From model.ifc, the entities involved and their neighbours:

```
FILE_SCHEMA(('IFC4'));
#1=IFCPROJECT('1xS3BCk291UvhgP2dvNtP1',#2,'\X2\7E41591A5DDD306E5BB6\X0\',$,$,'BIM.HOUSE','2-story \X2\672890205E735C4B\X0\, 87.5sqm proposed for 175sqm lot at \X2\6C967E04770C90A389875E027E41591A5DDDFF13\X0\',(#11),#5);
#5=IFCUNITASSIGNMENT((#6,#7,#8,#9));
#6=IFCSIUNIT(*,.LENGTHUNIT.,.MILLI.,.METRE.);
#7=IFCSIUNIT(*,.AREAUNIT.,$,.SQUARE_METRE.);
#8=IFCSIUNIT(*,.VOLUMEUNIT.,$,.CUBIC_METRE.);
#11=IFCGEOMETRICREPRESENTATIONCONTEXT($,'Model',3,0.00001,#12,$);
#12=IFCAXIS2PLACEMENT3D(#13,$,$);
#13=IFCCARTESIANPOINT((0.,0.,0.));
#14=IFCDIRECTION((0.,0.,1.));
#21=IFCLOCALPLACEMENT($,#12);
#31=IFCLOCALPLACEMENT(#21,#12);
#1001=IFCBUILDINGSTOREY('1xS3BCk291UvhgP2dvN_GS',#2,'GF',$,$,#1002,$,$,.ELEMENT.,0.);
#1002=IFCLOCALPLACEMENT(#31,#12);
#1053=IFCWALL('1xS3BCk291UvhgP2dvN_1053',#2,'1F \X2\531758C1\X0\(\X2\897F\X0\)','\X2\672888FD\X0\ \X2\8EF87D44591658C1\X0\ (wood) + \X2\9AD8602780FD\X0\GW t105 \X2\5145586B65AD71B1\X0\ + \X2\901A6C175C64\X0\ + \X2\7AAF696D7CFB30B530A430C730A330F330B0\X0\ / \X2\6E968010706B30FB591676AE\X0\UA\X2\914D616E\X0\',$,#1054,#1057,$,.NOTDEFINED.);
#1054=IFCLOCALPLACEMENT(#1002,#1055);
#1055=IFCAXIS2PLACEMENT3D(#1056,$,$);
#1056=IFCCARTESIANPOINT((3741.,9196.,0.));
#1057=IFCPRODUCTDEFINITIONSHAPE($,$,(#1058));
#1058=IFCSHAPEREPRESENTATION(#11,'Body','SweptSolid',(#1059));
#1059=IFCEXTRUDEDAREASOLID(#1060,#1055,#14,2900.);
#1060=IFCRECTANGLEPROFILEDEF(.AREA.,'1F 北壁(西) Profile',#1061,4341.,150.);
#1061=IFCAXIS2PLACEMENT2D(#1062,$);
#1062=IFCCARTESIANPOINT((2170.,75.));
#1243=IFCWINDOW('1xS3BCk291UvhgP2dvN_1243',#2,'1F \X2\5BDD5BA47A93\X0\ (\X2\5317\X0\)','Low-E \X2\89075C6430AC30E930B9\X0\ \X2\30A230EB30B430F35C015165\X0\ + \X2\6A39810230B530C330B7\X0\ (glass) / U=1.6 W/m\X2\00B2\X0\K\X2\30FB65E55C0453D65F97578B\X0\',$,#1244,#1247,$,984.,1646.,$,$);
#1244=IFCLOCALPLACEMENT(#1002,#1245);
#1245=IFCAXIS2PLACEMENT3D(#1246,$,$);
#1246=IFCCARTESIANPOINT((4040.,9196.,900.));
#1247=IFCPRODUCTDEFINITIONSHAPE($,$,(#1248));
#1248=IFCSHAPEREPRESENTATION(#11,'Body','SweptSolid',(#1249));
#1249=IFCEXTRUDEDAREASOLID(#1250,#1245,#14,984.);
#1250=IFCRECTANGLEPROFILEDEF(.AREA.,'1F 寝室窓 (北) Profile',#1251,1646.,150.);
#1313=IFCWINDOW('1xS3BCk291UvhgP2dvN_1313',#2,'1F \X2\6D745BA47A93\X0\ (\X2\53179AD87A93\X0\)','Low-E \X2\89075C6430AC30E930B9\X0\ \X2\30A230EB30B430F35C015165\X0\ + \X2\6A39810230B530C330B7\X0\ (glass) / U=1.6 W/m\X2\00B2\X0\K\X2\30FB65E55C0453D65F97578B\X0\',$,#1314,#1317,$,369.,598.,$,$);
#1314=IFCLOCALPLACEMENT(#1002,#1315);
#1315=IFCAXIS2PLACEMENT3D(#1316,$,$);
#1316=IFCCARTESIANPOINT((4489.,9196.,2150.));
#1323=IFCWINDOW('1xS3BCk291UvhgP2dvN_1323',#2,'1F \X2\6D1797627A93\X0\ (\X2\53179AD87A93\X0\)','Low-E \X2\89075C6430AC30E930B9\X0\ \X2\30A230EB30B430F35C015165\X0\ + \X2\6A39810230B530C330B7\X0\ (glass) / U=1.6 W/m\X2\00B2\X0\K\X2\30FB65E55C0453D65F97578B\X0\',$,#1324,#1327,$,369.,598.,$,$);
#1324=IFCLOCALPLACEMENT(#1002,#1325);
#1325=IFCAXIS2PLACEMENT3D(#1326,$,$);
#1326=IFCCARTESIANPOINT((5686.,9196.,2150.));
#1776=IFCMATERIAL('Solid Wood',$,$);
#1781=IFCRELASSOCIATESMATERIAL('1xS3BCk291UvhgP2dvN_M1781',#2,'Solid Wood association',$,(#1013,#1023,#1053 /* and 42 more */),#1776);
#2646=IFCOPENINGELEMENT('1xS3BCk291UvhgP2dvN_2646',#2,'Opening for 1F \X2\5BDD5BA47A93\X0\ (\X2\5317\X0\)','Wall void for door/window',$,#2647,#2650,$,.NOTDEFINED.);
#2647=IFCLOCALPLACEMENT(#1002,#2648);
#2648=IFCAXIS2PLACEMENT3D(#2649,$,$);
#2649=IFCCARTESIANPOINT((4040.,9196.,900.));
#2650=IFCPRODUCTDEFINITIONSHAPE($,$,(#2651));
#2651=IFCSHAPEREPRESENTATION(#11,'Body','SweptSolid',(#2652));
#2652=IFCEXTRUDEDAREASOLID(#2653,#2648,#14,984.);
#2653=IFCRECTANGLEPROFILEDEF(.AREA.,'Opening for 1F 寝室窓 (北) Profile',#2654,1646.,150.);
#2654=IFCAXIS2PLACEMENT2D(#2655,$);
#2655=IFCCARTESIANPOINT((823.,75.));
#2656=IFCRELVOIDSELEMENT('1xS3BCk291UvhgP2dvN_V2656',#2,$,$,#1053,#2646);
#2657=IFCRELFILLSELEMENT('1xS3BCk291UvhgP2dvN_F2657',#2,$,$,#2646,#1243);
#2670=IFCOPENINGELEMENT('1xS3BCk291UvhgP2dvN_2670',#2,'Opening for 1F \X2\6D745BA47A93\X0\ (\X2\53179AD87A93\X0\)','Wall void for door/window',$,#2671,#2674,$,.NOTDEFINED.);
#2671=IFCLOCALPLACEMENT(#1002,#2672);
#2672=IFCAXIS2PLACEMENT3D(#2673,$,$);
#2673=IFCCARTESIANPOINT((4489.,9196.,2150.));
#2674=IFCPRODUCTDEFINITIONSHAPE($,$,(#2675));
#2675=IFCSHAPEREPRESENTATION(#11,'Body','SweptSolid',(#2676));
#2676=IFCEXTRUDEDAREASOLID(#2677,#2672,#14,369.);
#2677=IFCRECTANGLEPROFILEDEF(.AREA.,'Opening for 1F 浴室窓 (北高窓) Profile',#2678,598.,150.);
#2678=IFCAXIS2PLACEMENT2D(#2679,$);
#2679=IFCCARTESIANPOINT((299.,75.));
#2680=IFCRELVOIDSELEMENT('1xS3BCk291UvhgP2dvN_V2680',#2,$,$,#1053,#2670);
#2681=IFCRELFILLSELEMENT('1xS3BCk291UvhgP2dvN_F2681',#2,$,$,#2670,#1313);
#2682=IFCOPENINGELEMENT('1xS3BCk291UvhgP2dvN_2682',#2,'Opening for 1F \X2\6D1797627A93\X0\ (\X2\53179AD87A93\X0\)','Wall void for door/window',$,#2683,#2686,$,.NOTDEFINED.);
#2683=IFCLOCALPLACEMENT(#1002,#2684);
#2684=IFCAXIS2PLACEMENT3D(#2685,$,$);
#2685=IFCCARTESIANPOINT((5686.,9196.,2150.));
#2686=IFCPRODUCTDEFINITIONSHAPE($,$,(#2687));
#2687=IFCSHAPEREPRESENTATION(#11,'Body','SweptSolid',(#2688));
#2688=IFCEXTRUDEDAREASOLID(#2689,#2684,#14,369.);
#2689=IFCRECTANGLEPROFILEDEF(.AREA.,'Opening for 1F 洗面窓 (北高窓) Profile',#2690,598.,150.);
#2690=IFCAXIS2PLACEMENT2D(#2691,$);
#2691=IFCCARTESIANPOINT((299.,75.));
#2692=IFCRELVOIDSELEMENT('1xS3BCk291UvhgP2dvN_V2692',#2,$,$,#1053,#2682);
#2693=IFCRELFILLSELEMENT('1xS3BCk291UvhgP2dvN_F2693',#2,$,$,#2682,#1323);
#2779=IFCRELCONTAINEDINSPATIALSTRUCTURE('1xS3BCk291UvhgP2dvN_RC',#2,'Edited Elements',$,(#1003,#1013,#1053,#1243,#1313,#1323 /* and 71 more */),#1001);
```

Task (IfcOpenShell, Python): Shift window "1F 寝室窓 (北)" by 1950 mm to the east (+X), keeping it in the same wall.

```python
import ifcopenshell
import ifcopenshell.api.geometry
import ifcopenshell.util.placement

model = ifcopenshell.open("model.ifc")

window = model.by_guid("1xS3BCk291UvhgP2dvN_1243")
opening = window.FillsVoids[0].RelatingOpeningElement
wall = opening.VoidsElements[0].RelatingBuildingElement

wall_matrix = ifcopenshell.util.placement.get_local_placement(wall.ObjectPlacement)
shift = wall_matrix[:3, 0] * 1950.0
before = ifcopenshell.util.placement.get_local_placement(window.ObjectPlacement)[:3, 3].copy()

# The window is not placed relative to its opening, so move both.
for product in (opening, window):
    matrix = ifcopenshell.util.placement.get_local_placement(product.ObjectPlacement)
    matrix[:3, 3] += shift
    ifcopenshell.api.geometry.edit_object_placement(model, product=product, matrix=matrix, is_si=False)

after = ifcopenshell.util.placement.get_local_placement(window.ObjectPlacement)[:3, 3]
print("window moved by", (after - before).round(3) + 0.0)

model.write("model_edited.ifc")
```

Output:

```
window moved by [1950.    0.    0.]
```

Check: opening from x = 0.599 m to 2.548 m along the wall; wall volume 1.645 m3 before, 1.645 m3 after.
